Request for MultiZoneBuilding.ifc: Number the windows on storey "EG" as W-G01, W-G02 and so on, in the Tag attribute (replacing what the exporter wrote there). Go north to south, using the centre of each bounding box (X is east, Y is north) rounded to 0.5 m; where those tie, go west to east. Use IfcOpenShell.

First a look at what the model holds.

```python
import ifcopenshell
import ifcopenshell.util.element
import ifcopenshell.util.placement

model = ifcopenshell.open("MultiZoneBuilding.ifc")
print(model.schema)
storey = next(s for s in model.by_type("IfcBuildingStorey") if s.Name == "EG")
windows = [e for e in ifcopenshell.util.element.get_decomposition(storey) if e.is_a("IfcWindow")]
for e in sorted(windows, key=lambda e: e.id()):
    origin = ifcopenshell.util.placement.get_local_placement(e.ObjectPlacement)[:3, 3]
    print(e.id(), e.Tag, e.Name, origin.round(2) + 0.0, sep=" | ")
```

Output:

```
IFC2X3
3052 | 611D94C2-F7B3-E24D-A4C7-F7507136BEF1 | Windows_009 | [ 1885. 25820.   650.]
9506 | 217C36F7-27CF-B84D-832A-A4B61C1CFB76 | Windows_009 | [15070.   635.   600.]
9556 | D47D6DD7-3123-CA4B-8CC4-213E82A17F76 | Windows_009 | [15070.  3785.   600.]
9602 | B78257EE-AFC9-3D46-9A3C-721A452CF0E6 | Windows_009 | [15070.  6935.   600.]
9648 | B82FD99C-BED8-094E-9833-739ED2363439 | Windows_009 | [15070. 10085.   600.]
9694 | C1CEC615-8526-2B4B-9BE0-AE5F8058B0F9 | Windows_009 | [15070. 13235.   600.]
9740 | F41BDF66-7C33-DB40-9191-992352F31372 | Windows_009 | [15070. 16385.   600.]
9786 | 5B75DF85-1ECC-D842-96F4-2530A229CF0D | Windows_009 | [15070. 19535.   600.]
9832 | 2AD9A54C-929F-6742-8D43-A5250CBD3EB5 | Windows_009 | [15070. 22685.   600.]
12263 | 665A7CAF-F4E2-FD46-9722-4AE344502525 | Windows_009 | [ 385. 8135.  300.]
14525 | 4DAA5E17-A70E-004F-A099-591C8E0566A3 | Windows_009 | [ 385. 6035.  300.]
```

```python
import ifcopenshell
import ifcopenshell.geom
import ifcopenshell.util.element
import ifcopenshell.util.shape

model = ifcopenshell.open("MultiZoneBuilding.ifc")
settings = ifcopenshell.geom.settings()
settings.set("use-world-coords", True)


def centre(element):
    shape = ifcopenshell.geom.create_shape(settings, element)
    return ifcopenshell.util.shape.get_bbox_centroid(shape.geometry)


storey = next(s for s in model.by_type("IfcBuildingStorey") if s.Name == "EG")
windows = [e for e in ifcopenshell.util.element.get_decomposition(storey) if e.is_a("IfcWindow")]

# Insertion points can sit at a corner or the storey origin, so sort by the geometry (in metres).
centres = {e: centre(e) for e in windows}
windows.sort(key=lambda e: (-round(centres[e][1] / 0.5), centres[e][0]))

for i, e in enumerate(windows, start=1):
    number = f"W-G{i:02d}"
    e.Tag = number
    print(e.id(), number)

model.write("MultiZoneBuilding_updated.ifc")
```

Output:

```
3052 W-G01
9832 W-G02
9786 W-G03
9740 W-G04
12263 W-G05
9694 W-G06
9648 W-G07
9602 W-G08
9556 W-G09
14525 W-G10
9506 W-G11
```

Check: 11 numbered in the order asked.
